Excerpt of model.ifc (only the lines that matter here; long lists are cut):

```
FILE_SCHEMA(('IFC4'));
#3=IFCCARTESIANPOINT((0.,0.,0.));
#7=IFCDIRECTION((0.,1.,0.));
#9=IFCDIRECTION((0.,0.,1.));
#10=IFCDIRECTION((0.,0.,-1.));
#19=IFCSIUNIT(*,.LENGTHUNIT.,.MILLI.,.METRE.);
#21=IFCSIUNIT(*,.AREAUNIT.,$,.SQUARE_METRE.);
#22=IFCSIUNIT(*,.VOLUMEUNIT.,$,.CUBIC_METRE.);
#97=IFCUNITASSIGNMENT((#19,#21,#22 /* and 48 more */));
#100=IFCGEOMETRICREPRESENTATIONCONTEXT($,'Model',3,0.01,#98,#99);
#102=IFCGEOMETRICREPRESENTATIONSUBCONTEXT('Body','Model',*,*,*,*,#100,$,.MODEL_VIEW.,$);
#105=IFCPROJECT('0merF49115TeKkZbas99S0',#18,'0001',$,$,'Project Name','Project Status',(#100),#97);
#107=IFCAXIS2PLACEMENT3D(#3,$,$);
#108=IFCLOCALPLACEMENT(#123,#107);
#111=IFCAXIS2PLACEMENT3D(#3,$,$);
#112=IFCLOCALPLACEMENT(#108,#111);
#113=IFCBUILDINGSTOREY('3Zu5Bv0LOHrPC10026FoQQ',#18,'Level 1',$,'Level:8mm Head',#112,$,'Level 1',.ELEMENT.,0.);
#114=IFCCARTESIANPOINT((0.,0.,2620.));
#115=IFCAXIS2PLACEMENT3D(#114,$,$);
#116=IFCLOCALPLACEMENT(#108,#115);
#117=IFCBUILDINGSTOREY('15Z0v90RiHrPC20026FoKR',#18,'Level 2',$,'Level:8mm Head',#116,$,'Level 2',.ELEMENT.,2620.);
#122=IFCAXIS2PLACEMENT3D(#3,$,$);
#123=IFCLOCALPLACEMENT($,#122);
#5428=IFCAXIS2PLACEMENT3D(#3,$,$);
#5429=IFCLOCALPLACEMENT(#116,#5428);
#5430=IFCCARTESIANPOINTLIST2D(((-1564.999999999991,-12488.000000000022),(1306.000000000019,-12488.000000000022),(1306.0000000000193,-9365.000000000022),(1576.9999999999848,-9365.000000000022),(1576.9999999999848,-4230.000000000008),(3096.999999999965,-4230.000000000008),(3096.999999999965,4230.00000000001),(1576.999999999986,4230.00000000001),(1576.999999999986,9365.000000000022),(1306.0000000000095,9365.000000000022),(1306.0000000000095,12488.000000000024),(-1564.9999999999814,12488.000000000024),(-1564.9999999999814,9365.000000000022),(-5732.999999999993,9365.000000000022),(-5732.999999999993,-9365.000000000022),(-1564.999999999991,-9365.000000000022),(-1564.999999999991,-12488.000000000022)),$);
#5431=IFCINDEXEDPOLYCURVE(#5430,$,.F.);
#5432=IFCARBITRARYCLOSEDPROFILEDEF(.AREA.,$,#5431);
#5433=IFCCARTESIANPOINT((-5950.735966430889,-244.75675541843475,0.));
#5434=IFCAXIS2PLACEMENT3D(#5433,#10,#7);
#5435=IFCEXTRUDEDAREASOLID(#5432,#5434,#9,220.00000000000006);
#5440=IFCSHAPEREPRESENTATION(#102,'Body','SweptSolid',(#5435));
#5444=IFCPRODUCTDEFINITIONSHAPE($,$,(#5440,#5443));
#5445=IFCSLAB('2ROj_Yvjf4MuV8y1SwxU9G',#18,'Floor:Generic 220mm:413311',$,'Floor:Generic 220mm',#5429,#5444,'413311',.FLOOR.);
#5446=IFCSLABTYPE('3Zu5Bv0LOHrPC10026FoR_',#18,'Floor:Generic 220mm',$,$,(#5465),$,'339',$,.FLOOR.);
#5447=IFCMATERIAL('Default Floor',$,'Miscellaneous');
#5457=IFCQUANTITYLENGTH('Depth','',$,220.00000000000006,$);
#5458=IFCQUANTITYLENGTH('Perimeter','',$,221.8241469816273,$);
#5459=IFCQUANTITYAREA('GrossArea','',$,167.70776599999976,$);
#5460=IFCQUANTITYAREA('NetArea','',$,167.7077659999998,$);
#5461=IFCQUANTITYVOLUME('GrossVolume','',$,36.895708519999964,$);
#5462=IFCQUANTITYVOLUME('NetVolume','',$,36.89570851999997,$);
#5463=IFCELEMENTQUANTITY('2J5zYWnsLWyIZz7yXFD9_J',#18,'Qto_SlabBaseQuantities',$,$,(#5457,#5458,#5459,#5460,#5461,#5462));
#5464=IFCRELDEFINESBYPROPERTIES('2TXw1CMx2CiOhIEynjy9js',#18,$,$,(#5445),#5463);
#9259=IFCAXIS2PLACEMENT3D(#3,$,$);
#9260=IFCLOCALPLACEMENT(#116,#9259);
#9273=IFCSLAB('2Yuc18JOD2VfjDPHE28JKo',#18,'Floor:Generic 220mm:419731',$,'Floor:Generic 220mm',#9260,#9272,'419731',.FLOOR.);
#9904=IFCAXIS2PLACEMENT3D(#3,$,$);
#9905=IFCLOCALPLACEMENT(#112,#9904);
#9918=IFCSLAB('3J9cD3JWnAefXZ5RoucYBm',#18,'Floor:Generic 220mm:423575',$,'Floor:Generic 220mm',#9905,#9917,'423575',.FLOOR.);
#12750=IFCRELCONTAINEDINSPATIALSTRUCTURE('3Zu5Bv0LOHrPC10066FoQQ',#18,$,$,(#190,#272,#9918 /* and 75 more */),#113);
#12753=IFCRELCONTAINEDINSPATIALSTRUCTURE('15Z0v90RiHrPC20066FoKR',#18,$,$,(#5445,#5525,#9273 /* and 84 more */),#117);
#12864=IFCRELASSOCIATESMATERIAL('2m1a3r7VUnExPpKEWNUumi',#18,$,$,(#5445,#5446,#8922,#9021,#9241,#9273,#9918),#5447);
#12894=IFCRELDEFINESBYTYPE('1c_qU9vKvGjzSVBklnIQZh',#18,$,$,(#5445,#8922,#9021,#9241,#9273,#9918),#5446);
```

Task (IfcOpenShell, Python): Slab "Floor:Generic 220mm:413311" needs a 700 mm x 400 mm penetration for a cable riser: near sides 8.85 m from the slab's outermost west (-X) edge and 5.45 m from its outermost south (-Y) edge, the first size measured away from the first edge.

```python
import numpy as np
import ifcopenshell
import ifcopenshell.api.feature
import ifcopenshell.api.geometry
import ifcopenshell.api.pset
import ifcopenshell.api.root
import ifcopenshell.geom
import ifcopenshell.util.element
import ifcopenshell.util.placement
import ifcopenshell.util.representation
import ifcopenshell.util.shape
import ifcopenshell.util.unit

model = ifcopenshell.open("model.ifc")
unit_scale = ifcopenshell.util.unit.calculate_unit_scale(model)
area_scale = ifcopenshell.util.unit.calculate_unit_scale(model, "AREAUNIT")
volume_scale = ifcopenshell.util.unit.calculate_unit_scale(model, "VOLUMEUNIT")
settings = ifcopenshell.geom.settings()


def volume(element):
    """Net volume in cubic metres, openings subtracted."""
    shape = ifcopenshell.geom.create_shape(settings, element)
    return ifcopenshell.util.shape.get_volume(shape.geometry)


slab = model.by_guid("2ROj_Yvjf4MuV8y1SwxU9G")
before = volume(slab)

# Extent in the slab's own axes, in metres. The edges named are its -X and -Y sides.
slab_shape = ifcopenshell.geom.create_shape(settings, slab)
vertices = ifcopenshell.util.shape.get_vertices(slab_shape.geometry)
x_min, y_min, bottom = vertices.min(axis=0)
top = vertices[:, 2].max()

opening = ifcopenshell.api.root.create_entity(model, ifc_class="IfcOpeningElement", name="Cable riser opening", predefined_type="OPENING")
context = ifcopenshell.util.representation.get_context(model, "Model", "Body", "MODEL_VIEW")
width, depth = 0.7, 0.4
outline = [(0.0, 0.0), (width, 0.0), (width, depth), (0.0, depth), (0.0, 0.0)]
# Overshoot both faces by 50 mm so the cut is clean.
shape = ifcopenshell.api.geometry.add_slab_representation(
    model, context=context, depth=top - bottom + 0.1, polyline=outline
)
ifcopenshell.api.geometry.assign_representation(model, product=opening, representation=shape)

matrix = ifcopenshell.util.placement.get_local_placement(slab.ObjectPlacement)
matrix[:, 3] = matrix @ np.append(np.array([x_min + 8.85, y_min + 5.45, bottom - 0.05]) / unit_scale, 1.0)
ifcopenshell.api.geometry.edit_object_placement(model, product=opening, matrix=matrix, is_si=False)
ifcopenshell.api.feature.add_feature(model, feature=opening, element=slab)

after = volume(slab)

# Update the slab's stored quantities.
qto = model.by_id(ifcopenshell.util.element.get_pset(slab, "Qto_SlabBaseQuantities", should_inherit=False)["id"])
ifcopenshell.api.pset.edit_qto(model, qto=qto, properties={
    "NetArea": after / (top - bottom) / area_scale,
    "NetVolume": after / volume_scale,
})

print(f"slab volume {before:.3f} -> {after:.3f} m3")

model.write("model_edited.ifc")
```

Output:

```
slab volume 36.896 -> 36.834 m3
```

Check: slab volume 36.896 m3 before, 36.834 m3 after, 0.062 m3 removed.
